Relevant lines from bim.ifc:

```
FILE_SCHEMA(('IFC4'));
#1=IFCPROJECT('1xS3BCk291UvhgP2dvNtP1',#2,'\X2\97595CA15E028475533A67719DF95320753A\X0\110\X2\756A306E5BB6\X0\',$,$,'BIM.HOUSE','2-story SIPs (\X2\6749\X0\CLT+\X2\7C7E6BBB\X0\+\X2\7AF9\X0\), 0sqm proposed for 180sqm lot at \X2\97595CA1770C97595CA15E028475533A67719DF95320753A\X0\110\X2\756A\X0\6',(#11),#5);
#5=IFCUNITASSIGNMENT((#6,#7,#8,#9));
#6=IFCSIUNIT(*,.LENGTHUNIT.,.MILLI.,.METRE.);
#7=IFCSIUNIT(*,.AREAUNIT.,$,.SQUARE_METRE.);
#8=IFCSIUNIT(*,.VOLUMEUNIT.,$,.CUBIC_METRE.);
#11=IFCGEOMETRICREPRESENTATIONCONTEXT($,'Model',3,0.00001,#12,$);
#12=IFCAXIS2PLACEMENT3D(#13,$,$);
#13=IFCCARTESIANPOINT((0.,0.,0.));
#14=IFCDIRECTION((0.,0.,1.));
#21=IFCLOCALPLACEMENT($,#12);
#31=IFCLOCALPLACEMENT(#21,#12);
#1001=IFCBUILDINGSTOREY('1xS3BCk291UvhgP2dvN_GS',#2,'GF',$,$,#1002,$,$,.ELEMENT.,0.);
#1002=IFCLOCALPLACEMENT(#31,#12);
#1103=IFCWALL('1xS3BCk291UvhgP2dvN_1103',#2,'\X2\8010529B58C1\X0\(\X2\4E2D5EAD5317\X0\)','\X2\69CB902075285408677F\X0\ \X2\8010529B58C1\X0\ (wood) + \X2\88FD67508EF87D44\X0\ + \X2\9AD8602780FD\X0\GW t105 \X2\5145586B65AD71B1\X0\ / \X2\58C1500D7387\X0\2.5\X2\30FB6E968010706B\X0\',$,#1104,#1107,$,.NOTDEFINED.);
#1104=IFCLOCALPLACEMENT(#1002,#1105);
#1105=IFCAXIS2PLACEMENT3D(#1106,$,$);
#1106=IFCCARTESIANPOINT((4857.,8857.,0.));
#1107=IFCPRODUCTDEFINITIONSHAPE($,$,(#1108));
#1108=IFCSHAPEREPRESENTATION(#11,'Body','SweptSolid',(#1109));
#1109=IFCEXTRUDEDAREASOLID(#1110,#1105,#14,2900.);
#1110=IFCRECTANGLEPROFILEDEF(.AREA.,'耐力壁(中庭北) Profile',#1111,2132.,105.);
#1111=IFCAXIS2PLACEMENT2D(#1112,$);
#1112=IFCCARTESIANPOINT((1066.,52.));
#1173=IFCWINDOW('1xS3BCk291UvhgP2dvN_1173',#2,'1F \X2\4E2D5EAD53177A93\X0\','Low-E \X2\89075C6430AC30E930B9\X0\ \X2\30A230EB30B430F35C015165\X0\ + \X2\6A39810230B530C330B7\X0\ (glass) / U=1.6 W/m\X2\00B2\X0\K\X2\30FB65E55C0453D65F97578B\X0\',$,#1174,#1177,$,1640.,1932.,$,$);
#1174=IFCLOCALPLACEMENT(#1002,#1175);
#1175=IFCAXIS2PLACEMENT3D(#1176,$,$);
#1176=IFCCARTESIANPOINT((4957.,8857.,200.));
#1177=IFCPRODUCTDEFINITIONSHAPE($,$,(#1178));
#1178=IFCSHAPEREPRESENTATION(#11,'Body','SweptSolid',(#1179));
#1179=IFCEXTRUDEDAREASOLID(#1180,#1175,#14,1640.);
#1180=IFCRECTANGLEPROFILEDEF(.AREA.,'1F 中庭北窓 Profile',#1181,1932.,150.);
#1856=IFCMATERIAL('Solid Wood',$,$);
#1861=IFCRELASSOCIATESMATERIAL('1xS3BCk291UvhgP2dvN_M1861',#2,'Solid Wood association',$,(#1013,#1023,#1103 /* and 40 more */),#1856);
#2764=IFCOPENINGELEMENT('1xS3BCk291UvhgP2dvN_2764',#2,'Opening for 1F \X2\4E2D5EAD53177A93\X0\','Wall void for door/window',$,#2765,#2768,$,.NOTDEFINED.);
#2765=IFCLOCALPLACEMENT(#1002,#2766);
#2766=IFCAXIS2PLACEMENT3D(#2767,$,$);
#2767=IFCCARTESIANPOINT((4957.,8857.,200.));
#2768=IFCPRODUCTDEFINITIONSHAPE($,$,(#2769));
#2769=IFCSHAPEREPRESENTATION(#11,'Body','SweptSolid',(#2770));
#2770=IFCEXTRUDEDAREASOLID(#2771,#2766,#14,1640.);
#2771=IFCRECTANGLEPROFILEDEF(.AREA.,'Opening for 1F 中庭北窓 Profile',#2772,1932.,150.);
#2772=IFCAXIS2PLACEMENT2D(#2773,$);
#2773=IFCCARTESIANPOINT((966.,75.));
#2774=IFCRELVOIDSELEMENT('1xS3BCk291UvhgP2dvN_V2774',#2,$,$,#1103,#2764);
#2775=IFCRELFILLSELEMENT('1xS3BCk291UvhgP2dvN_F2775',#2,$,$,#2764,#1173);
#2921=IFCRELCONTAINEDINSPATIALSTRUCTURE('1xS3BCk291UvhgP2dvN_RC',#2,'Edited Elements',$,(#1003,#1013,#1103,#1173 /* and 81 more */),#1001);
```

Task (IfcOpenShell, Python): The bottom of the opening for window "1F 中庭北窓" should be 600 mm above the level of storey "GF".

```python
import numpy as np
import ifcopenshell
import ifcopenshell.api.geometry
import ifcopenshell.geom
import ifcopenshell.util.element
import ifcopenshell.util.placement
import ifcopenshell.util.shape
import ifcopenshell.util.unit

model = ifcopenshell.open("bim.ifc")
unit_scale = ifcopenshell.util.unit.calculate_unit_scale(model)

window = model.by_guid("1xS3BCk291UvhgP2dvN_1173")
opening = window.FillsVoids[0].RelatingOpeningElement
storey = ifcopenshell.util.element.get_container(window, ifc_class="IfcBuildingStorey")
level = ifcopenshell.util.placement.get_local_placement(storey.ObjectPlacement)[2, 3]

# The opening's origin need not be at the sill, so measure its lowest point.
shape = ifcopenshell.geom.create_shape(ifcopenshell.geom.settings(), opening)
bottom = ifcopenshell.util.shape.get_shape_bottom_elevation(shape, shape.geometry) / unit_scale
dz = level + 600.0 - bottom

shift = np.array([0.0, 0.0, dz])
# The window is not placed relative to its opening, so move both.
for product in (opening, window):
    matrix = ifcopenshell.util.placement.get_local_placement(product.ObjectPlacement)
    matrix[:3, 3] += shift
    ifcopenshell.api.geometry.edit_object_placement(model, product=product, matrix=matrix, is_si=False)

print(f"moved by {dz * unit_scale:+.3f} m")

model.write("bim_rev.ifc")
```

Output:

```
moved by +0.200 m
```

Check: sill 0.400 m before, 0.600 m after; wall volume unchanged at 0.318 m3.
